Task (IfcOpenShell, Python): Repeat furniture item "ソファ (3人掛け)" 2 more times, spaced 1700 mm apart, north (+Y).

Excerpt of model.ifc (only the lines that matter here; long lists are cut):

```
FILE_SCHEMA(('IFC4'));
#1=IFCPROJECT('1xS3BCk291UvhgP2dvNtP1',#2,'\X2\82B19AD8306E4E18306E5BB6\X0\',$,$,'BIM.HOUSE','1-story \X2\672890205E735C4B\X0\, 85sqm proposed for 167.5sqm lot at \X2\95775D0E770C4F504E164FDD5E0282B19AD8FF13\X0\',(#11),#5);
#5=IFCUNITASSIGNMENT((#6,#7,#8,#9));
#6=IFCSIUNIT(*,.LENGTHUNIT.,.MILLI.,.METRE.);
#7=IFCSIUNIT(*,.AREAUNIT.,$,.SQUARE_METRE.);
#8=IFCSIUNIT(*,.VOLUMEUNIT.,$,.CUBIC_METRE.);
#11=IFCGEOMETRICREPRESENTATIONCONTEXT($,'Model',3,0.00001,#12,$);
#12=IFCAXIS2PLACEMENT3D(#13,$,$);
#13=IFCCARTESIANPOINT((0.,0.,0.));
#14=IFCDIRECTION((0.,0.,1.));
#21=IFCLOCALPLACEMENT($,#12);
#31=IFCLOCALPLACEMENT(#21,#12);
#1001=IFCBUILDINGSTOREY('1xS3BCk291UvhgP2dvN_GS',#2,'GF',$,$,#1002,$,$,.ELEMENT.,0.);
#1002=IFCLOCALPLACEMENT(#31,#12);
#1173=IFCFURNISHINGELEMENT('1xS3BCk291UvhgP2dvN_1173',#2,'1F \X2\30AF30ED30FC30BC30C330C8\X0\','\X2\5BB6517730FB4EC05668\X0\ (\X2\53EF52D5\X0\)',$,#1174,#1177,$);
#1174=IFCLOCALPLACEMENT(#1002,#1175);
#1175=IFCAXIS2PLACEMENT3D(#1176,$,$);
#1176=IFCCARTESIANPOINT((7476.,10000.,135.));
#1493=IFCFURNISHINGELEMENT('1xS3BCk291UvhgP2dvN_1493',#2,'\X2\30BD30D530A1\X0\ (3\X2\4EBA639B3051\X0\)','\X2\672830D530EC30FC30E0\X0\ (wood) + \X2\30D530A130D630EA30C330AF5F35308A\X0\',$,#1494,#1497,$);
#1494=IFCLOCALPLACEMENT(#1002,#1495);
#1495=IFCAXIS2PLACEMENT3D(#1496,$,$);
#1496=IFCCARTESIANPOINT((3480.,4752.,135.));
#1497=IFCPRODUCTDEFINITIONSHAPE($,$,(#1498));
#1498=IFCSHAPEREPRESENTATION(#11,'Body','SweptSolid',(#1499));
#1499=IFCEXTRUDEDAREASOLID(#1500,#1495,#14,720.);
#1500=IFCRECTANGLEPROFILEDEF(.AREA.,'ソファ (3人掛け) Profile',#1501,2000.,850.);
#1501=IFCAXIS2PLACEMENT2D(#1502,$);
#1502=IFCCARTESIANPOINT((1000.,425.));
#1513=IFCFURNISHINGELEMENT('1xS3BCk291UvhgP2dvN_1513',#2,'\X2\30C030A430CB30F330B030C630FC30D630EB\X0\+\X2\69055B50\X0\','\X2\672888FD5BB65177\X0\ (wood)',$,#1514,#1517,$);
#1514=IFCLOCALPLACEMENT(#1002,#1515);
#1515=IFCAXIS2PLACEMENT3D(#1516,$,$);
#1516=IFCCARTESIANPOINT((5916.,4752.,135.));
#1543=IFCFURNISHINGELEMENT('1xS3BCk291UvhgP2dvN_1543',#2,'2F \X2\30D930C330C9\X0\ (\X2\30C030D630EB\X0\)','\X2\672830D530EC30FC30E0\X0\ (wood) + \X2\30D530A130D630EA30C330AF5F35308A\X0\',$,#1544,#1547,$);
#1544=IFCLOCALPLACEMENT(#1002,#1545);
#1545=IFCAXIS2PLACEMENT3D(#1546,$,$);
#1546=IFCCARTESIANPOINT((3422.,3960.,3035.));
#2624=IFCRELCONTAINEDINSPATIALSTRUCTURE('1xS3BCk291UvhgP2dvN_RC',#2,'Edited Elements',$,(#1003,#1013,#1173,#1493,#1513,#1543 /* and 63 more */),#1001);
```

```python
import numpy as np
import ifcopenshell
import ifcopenshell.api.geometry
import ifcopenshell.api.root
import ifcopenshell.util.element
import ifcopenshell.util.placement

model = ifcopenshell.open("model.ifc")


def reuse_history(source, copy):
    """copy_class also copies each property set's owner history, people and application; keep the originals."""
    for rel in copy.IsDefinedBy:
        if rel.is_a("IfcRelDefinesByProperties") and (history := rel.RelatingPropertyDefinition.OwnerHistory):
            rel.RelatingPropertyDefinition.OwnerHistory = source.OwnerHistory
            ifcopenshell.util.element.remove_deep2(model, history)


source = model.by_guid("1xS3BCk291UvhgP2dvN_1493")
base = ifcopenshell.util.placement.get_local_placement(source.ObjectPlacement)
step = np.array([0.0, 1.0, 0.0]) * 1700.0

for i in range(1, 3):
    copy = ifcopenshell.api.root.copy_class(model, product=source)
    copy.Representation = ifcopenshell.util.element.copy_deep(
        model, source.Representation, exclude=["IfcGeometricRepresentationContext", "IfcRepresentationMap"]
    )
    reuse_history(source, copy)
    matrix = base.copy()
    matrix[:3, 3] += i * step
    print("added at", matrix[:3, 3].round(3) + 0.0)
    ifcopenshell.api.geometry.edit_object_placement(model, product=copy, matrix=matrix, is_si=False)

model.write("model_updated.ifc")
```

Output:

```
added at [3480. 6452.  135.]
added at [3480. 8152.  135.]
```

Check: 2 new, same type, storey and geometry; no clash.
